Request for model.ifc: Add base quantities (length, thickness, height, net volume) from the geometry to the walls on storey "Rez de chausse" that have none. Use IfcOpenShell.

First a look at what the model holds.

```python
import ifcopenshell
import ifcopenshell.util.element
import ifcopenshell.util.unit

model = ifcopenshell.open("model.ifc")
print(model.schema)
for unit_type in ("LENGTHUNIT", "AREAUNIT", "VOLUMEUNIT"):
    print(unit_type, ifcopenshell.util.unit.calculate_unit_scale(model, unit_type))
storey = next(s for s in model.by_type("IfcBuildingStorey") if s.Name == 'Rez de chauss\x8ee')
walls = [e for e in ifcopenshell.util.element.get_decomposition(storey) if e.is_a("IfcWall")]
for e in sorted(walls, key=lambda e: e.id()):
    print(e.id(), e.is_a(), e.Name, list(ifcopenshell.util.element.get_psets(e, qtos_only=True)), sep=" | ")
```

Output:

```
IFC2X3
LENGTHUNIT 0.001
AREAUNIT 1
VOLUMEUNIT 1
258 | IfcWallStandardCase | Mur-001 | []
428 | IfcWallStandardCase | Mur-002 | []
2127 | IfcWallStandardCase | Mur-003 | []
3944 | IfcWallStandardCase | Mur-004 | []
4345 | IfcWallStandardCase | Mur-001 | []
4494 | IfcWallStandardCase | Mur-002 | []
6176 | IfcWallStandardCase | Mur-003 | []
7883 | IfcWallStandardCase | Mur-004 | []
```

```python
import ifcopenshell
import ifcopenshell.api.pset
import ifcopenshell.geom
import ifcopenshell.util.element
import ifcopenshell.util.shape
import ifcopenshell.util.unit

model = ifcopenshell.open("model.ifc")
unit_scale = ifcopenshell.util.unit.calculate_unit_scale(model)
volume_scale = ifcopenshell.util.unit.calculate_unit_scale(model, "VOLUMEUNIT")
settings = ifcopenshell.geom.settings()

storey = next(s for s in model.by_type("IfcBuildingStorey") if s.Name == 'Rez de chauss\x8ee')
walls = [e for e in ifcopenshell.util.element.get_decomposition(storey) if e.is_a("IfcWall")]

for e in sorted(walls, key=lambda e: e.id()):
    if ifcopenshell.util.element.get_psets(e, qtos_only=True, should_inherit=False):
        continue
    # Geometry comes back in metres, in the element's own axes.
    shape = ifcopenshell.geom.create_shape(settings, e)
    values = {
        "Length": ifcopenshell.util.shape.get_x(shape.geometry) / unit_scale,
        "Width": ifcopenshell.util.shape.get_y(shape.geometry) / unit_scale,
        "Height": ifcopenshell.util.shape.get_z(shape.geometry) / unit_scale,
        "NetVolume": ifcopenshell.util.shape.get_volume(shape.geometry) / volume_scale,
    }
    qto = ifcopenshell.api.pset.add_qto(model, product=e, name="BaseQuantities")
    ifcopenshell.api.pset.edit_qto(model, qto=qto, properties=values)
    print(e.id(), {k: round(v, 3) for k, v in values.items()})

model.write("model-out.ifc")
```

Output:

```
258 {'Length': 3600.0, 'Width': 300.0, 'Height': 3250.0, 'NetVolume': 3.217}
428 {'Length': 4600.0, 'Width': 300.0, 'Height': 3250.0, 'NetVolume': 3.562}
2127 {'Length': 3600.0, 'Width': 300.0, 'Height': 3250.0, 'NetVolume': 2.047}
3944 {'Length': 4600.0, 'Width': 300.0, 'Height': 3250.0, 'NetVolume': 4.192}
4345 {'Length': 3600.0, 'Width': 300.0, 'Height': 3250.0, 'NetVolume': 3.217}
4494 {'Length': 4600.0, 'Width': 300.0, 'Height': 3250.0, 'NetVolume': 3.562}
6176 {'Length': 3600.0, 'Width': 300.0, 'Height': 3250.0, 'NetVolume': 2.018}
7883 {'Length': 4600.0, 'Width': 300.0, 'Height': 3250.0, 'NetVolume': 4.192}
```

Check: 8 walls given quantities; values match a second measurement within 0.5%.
